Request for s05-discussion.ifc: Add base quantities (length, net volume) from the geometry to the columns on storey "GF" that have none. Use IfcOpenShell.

First a look at what the model holds.

```python
import ifcopenshell
import ifcopenshell.util.element
import ifcopenshell.util.unit

model = ifcopenshell.open("s05-discussion.ifc")
print(model.schema)
for unit_type in ("LENGTHUNIT", "AREAUNIT", "VOLUMEUNIT"):
    print(unit_type, ifcopenshell.util.unit.calculate_unit_scale(model, unit_type))
storey = next(s for s in model.by_type("IfcBuildingStorey") if s.Name == "GF")
columns = [e for e in ifcopenshell.util.element.get_decomposition(storey) if e.is_a("IfcColumn")]
for e in sorted(columns, key=lambda e: e.id()):
    print(e.id(), e.is_a(), e.Name, list(ifcopenshell.util.element.get_psets(e, qtos_only=True)), sep=" | ")
```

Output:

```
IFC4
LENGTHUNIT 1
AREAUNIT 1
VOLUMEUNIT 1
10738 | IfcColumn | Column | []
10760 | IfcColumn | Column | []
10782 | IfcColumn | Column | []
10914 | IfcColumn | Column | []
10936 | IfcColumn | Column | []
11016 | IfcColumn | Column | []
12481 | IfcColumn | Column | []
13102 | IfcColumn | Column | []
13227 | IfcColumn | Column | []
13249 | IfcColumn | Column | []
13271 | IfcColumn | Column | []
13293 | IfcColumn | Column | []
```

```python
import ifcopenshell
import ifcopenshell.api.pset
import ifcopenshell.geom
import ifcopenshell.util.element
import ifcopenshell.util.shape
import ifcopenshell.util.unit

model = ifcopenshell.open("s05-discussion.ifc")
unit_scale = ifcopenshell.util.unit.calculate_unit_scale(model)
volume_scale = ifcopenshell.util.unit.calculate_unit_scale(model, "VOLUMEUNIT")
settings = ifcopenshell.geom.settings()

storey = next(s for s in model.by_type("IfcBuildingStorey") if s.Name == "GF")
columns = [e for e in ifcopenshell.util.element.get_decomposition(storey) if e.is_a("IfcColumn")]

for e in sorted(columns, key=lambda e: e.id()):
    if ifcopenshell.util.element.get_psets(e, qtos_only=True, should_inherit=False):
        continue
    # Geometry comes back in metres, in the element's own axes.
    shape = ifcopenshell.geom.create_shape(settings, e)
    values = {
        "Length": ifcopenshell.util.shape.get_z(shape.geometry) / unit_scale,
        "NetVolume": ifcopenshell.util.shape.get_volume(shape.geometry) / volume_scale,
    }
    qto = ifcopenshell.api.pset.add_qto(model, product=e, name="Qto_ColumnBaseQuantities")
    ifcopenshell.api.pset.edit_qto(model, qto=qto, properties=values)
    print(e.id(), {k: round(v, 3) for k, v in values.items()})

model.write("s05-discussion-out.ifc")
```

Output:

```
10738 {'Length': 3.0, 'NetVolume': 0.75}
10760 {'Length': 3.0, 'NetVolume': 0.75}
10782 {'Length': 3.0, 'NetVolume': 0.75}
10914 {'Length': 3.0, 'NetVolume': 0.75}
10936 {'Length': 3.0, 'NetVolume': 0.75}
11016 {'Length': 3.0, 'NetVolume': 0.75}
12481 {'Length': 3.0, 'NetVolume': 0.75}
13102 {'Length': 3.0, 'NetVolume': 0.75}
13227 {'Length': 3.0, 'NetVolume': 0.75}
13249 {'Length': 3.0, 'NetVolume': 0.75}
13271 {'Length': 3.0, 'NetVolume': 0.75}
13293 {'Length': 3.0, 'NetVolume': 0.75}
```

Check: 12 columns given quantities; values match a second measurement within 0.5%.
